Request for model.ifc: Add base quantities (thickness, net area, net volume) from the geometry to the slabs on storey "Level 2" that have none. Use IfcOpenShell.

First a look at what the model holds.

```python
import ifcopenshell
import ifcopenshell.util.element
import ifcopenshell.util.unit

model = ifcopenshell.open("model.ifc")
print(model.schema)
for unit_type in ("LENGTHUNIT", "AREAUNIT", "VOLUMEUNIT"):
    print(unit_type, ifcopenshell.util.unit.calculate_unit_scale(model, unit_type))
storey = next(s for s in model.by_type("IfcBuildingStorey") if s.Name == "Level 2")
slabs = [e for e in ifcopenshell.util.element.get_decomposition(storey) if e.is_a("IfcSlab")]
for e in sorted(slabs, key=lambda e: e.id()):
    print(e.id(), e.is_a(), e.Name, list(ifcopenshell.util.element.get_psets(e, qtos_only=True)), sep=" | ")
```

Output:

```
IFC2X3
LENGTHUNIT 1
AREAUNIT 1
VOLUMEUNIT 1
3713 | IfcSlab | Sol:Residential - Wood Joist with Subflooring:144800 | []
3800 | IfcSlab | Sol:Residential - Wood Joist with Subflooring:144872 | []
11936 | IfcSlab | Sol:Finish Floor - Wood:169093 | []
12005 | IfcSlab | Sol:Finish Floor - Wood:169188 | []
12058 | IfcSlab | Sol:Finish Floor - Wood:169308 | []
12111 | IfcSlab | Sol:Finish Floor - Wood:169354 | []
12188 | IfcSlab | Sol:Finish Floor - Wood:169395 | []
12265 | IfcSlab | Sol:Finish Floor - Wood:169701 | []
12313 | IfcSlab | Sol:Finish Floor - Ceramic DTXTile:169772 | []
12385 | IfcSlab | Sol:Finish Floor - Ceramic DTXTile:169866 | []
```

```python
import ifcopenshell
import ifcopenshell.api.pset
import ifcopenshell.geom
import ifcopenshell.util.element
import ifcopenshell.util.shape
import ifcopenshell.util.unit

model = ifcopenshell.open("model.ifc")
unit_scale = ifcopenshell.util.unit.calculate_unit_scale(model)
area_scale = ifcopenshell.util.unit.calculate_unit_scale(model, "AREAUNIT")
volume_scale = ifcopenshell.util.unit.calculate_unit_scale(model, "VOLUMEUNIT")
settings = ifcopenshell.geom.settings()

storey = next(s for s in model.by_type("IfcBuildingStorey") if s.Name == "Level 2")
slabs = [e for e in ifcopenshell.util.element.get_decomposition(storey) if e.is_a("IfcSlab")]

for e in sorted(slabs, key=lambda e: e.id()):
    if ifcopenshell.util.element.get_psets(e, qtos_only=True, should_inherit=False):
        continue
    # Geometry comes back in metres, in the element's own axes.
    shape = ifcopenshell.geom.create_shape(settings, e)
    values = {
        "Width": ifcopenshell.util.shape.get_z(shape.geometry) / unit_scale,
        "NetArea": ifcopenshell.util.shape.get_footprint_area(shape.geometry) / area_scale,
        "NetVolume": ifcopenshell.util.shape.get_volume(shape.geometry) / volume_scale,
    }
    qto = ifcopenshell.api.pset.add_qto(model, product=e, name="BaseQuantities")
    ifcopenshell.api.pset.edit_qto(model, qto=qto, properties=values)
    print(e.id(), {k: round(v, 3) for k, v in values.items()})

model.write("model_rev.ifc")
```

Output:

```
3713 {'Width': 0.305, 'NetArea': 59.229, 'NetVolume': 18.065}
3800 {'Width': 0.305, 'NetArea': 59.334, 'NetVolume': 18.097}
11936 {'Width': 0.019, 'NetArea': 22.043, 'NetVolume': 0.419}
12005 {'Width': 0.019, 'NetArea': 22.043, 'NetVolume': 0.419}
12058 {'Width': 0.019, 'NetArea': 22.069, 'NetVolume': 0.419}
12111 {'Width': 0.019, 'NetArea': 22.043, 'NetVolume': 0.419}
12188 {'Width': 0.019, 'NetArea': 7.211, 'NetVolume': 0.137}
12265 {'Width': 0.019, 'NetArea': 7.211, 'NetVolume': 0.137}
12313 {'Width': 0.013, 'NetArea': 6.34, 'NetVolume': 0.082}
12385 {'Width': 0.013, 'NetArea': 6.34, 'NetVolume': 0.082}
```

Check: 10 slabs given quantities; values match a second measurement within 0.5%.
